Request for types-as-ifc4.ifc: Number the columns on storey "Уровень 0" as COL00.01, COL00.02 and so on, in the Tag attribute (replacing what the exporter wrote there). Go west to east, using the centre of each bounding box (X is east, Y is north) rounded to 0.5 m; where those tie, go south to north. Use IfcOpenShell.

First a look at what the model holds.

```python
import ifcopenshell
import ifcopenshell.util.element
import ifcopenshell.util.placement

model = ifcopenshell.open("types-as-ifc4.ifc")
print(model.schema)
storey = next(s for s in model.by_type("IfcBuildingStorey") if s.Name == "Уровень 0")
columns = [e for e in ifcopenshell.util.element.get_decomposition(storey) if e.is_a("IfcColumn")]
for e in sorted(columns, key=lambda e: e.id()):
    origin = ifcopenshell.util.placement.get_local_placement(e.ObjectPlacement)[:3, 3]
    print(e.id(), e.Tag, e.Name, origin.round(2) + 0.0, sep=" | ")
```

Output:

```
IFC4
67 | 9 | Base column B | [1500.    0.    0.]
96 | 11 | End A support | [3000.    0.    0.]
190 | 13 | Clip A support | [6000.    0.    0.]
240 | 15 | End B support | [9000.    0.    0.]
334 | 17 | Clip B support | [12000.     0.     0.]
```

```python
import ifcopenshell
import ifcopenshell.geom
import ifcopenshell.util.element
import ifcopenshell.util.shape

model = ifcopenshell.open("types-as-ifc4.ifc")
settings = ifcopenshell.geom.settings()
settings.set("use-world-coords", True)


def centre(element):
    shape = ifcopenshell.geom.create_shape(settings, element)
    return ifcopenshell.util.shape.get_bbox_centroid(shape.geometry)


storey = next(s for s in model.by_type("IfcBuildingStorey") if s.Name == "Уровень 0")
columns = [e for e in ifcopenshell.util.element.get_decomposition(storey) if e.is_a("IfcColumn")]

# Insertion points can sit at a corner or the storey origin, so sort by the geometry (in metres).
centres = {e: centre(e) for e in columns}
columns.sort(key=lambda e: (round(centres[e][0] / 0.5), centres[e][1]))

for i, e in enumerate(columns, start=1):
    number = f"COL00.{i:02d}"
    e.Tag = number
    print(e.id(), number)

model.write("types-as-ifc4_rev.ifc")
```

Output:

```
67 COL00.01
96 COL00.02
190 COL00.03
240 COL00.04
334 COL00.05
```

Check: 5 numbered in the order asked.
